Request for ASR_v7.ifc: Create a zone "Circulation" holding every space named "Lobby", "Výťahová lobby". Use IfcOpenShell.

First a look at what the model holds.

```python
import ifcopenshell

model = ifcopenshell.open("ASR_v7.ifc")
print(model.schema)
seen = {}
for space in model.by_type("IfcSpace"):
    seen[space.LongName] = seen.get(space.LongName, 0) + 1
for name, count in sorted(seen.items(), key=str):
    print(count, "x", name)
print("zones:", [z.Name for z in model.by_type("IfcZone")][:20])
```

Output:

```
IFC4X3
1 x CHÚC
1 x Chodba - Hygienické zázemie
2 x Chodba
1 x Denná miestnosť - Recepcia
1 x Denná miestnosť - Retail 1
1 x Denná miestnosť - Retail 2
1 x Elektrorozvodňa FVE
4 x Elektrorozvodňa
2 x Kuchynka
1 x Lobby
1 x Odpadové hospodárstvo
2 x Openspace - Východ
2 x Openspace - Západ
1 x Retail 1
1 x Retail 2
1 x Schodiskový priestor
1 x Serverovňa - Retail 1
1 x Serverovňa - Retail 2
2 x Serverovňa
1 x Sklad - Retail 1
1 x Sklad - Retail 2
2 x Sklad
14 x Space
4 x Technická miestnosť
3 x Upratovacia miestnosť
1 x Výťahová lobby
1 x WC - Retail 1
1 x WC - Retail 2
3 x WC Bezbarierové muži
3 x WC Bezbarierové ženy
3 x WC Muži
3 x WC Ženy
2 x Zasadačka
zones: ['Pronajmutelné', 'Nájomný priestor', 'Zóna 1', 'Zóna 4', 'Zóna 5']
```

```python
import ifcopenshell
import ifcopenshell.api.group
import ifcopenshell.api.root

model = ifcopenshell.open("ASR_v7.ifc")

names = {"Lobby", "Výťahová lobby"}
spaces = [s for s in model.by_type("IfcSpace") if s.LongName in names]

zone = ifcopenshell.api.root.create_entity(model, ifc_class="IfcZone", name="Circulation")
ifcopenshell.api.group.assign_group(model, products=spaces, group=zone)
print(len(spaces), "spaces in", zone.Name)

model.write("ASR_v7_rev.ifc")
```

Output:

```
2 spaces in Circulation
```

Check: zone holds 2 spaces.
